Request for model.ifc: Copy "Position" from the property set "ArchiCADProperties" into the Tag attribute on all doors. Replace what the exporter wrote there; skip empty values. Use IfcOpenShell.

First a look at what the model holds.

```python
import ifcopenshell
import ifcopenshell.util.element

model = ifcopenshell.open("model.ifc")
print(model.schema)
doors = model.by_type("IfcDoor")
print(len(doors), "doors")
for e in doors[:8]:
    source = ifcopenshell.util.element.get_pset(e, "ArchiCADProperties", "Position")
    target = e.Tag
    print(e.id(), repr(source), repr(target), sep=" | ")
```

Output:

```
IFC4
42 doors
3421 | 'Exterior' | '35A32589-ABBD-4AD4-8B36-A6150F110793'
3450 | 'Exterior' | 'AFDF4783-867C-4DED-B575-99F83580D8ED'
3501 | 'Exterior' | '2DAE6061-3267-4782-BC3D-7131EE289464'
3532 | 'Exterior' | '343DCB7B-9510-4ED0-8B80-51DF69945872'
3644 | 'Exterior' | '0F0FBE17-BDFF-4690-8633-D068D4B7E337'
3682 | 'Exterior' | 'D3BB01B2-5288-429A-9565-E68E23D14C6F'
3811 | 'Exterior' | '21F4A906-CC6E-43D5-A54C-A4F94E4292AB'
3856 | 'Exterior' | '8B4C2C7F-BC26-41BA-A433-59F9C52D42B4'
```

```python
import ifcopenshell
import ifcopenshell.util.element

model = ifcopenshell.open("model.ifc")

count = 0
for e in model.by_type("IfcDoor"):
    value = ifcopenshell.util.element.get_pset(e, "ArchiCADProperties", "Position")
    current = e.Tag
    if not value or not value.strip() or current == value:
        continue
    e.Tag = value
    count += 1

print(count, "doors updated")

model.write("model_rev.ifc")
```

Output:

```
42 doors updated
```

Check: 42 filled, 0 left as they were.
